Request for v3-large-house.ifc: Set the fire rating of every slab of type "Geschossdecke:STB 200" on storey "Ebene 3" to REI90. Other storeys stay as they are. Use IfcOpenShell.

First a look at what the model holds.

```python
import ifcopenshell
import ifcopenshell.util.element

model = ifcopenshell.open("v3-large-house.ifc")
print(model.schema)
storey = next(s for s in model.by_type("IfcBuildingStorey") if s.Name == "Ebene 3")
slabs = [e for e in ifcopenshell.util.element.get_decomposition(storey) if e.is_a("IfcSlab")]
seen = {}
for e in slabs:
    element_type = ifcopenshell.util.element.get_type(e)
    key = (element_type.Name if element_type != e and element_type else None, ifcopenshell.util.element.get_pset(e, "Pset_SlabCommon", "FireRating"))
    seen[key] = seen.get(key, 0) + 1
for (name, value), count in sorted(seen.items(), key=str):
    print(count, "x", name, "|", value)
```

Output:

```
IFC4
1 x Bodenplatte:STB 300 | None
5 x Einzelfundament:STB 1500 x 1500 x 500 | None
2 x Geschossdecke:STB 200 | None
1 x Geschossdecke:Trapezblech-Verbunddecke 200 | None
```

```python
import ifcopenshell
import ifcopenshell.api.pset
import ifcopenshell.util.element

model = ifcopenshell.open("v3-large-house.ifc")

storey = next(s for s in model.by_type("IfcBuildingStorey") if s.Name == "Ebene 3")
slabs = [e for e in ifcopenshell.util.element.get_decomposition(storey) if e.is_a("IfcSlab")]

count = 0
for e in slabs:
    element_type = ifcopenshell.util.element.get_type(e)
    if element_type in (None, e) or element_type.Name != "Geschossdecke:STB 200":
        continue
    # add_pset returns the element's existing set when there is one.
    pset = ifcopenshell.api.pset.add_pset(model, product=e, name="Pset_SlabCommon")
    ifcopenshell.api.pset.edit_pset(model, pset=pset, properties={"FireRating": "REI90"})
    count += 1

print(count, "slabs updated")

model.write("v3-large-house_updated.ifc")
```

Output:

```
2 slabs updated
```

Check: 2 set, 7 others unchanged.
